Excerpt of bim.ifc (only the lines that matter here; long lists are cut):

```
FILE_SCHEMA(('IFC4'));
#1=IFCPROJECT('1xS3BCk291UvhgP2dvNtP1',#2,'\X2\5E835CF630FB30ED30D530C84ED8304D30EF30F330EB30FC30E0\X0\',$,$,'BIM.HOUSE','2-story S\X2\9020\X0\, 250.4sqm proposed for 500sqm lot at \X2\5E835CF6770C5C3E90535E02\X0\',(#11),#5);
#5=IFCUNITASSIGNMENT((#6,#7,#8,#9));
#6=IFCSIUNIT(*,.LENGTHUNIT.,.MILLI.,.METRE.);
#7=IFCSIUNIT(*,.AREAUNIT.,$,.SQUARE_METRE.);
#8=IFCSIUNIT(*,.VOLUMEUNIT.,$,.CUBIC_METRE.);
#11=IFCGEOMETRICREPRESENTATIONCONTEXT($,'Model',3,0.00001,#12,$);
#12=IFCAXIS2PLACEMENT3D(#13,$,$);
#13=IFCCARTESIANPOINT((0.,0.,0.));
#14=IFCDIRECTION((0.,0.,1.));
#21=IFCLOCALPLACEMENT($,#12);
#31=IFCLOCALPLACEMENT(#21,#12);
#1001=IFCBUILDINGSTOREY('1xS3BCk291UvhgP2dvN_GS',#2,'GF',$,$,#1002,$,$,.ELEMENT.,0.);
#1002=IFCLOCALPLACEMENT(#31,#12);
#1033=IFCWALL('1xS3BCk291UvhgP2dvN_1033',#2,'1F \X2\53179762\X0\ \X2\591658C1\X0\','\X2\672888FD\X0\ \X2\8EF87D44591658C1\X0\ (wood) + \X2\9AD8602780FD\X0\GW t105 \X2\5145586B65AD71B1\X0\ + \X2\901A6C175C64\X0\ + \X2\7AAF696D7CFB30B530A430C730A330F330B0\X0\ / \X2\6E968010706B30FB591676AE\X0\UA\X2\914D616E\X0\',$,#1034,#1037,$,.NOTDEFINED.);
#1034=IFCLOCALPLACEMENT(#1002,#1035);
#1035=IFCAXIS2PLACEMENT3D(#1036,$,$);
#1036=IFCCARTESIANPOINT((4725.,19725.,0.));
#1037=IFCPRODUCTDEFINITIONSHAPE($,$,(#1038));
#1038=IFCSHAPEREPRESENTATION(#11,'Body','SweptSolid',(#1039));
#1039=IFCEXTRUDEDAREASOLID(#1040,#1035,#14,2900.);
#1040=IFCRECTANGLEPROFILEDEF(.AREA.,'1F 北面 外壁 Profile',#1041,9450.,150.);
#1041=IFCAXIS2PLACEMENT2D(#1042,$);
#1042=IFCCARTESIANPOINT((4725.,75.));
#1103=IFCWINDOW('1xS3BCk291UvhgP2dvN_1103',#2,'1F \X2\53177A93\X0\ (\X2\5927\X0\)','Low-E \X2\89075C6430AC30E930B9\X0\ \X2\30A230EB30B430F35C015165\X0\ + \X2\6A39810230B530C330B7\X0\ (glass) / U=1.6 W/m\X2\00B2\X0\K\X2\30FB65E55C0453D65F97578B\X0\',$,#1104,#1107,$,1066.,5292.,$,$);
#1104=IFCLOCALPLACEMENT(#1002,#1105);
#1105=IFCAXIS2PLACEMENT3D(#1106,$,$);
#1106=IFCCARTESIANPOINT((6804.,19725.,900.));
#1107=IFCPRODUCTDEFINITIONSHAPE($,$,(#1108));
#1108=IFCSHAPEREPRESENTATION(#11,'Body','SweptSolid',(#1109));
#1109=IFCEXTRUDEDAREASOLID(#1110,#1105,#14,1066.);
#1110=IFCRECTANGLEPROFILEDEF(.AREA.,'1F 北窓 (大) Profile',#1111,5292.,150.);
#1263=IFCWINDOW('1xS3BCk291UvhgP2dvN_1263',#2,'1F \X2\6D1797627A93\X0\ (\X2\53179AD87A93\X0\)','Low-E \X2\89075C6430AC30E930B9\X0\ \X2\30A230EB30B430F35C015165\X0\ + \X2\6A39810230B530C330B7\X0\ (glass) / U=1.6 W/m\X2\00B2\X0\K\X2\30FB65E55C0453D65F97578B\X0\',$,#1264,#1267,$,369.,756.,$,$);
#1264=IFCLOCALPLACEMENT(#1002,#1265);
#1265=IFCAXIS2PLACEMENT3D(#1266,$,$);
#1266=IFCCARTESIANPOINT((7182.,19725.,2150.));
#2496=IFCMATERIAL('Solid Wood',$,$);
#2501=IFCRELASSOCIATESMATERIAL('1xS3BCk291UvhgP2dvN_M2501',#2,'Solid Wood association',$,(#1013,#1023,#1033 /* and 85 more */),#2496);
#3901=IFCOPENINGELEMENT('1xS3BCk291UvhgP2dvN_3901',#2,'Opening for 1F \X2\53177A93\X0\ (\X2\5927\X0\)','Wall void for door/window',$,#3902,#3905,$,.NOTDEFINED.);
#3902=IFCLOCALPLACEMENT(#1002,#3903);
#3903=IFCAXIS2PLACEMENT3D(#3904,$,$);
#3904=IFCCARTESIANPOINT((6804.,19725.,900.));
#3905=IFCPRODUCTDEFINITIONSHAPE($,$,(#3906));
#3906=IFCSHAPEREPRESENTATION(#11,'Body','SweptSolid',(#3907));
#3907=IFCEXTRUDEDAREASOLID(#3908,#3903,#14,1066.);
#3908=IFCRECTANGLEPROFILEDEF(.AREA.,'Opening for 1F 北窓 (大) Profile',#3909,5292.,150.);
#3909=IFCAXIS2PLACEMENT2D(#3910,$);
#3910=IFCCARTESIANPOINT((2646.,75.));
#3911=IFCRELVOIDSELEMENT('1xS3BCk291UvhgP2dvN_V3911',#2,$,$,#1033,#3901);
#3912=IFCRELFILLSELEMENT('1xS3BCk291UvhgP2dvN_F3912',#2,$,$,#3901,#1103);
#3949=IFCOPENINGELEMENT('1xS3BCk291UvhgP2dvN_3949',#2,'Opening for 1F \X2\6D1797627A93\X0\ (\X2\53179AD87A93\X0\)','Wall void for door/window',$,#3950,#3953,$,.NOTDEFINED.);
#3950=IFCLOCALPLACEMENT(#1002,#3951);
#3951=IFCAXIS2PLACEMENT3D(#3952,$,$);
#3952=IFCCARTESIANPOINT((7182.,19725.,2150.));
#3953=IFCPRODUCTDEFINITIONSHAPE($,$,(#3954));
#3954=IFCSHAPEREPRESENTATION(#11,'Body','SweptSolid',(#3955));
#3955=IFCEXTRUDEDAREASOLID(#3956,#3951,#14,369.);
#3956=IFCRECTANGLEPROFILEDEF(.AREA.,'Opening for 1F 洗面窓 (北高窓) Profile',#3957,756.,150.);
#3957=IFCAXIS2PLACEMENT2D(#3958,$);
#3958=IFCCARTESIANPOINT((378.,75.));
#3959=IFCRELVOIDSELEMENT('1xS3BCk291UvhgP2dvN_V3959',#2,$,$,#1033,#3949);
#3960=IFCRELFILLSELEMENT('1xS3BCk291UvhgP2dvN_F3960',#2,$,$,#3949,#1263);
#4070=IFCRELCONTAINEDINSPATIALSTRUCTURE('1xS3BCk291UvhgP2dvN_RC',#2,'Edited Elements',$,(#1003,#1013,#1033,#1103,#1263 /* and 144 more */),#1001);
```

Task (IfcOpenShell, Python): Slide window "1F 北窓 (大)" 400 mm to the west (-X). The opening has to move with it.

```python
import ifcopenshell
import ifcopenshell.api.geometry
import ifcopenshell.util.placement

model = ifcopenshell.open("bim.ifc")

window = model.by_guid("1xS3BCk291UvhgP2dvN_1103")
opening = window.FillsVoids[0].RelatingOpeningElement
wall = opening.VoidsElements[0].RelatingBuildingElement

wall_matrix = ifcopenshell.util.placement.get_local_placement(wall.ObjectPlacement)
shift = wall_matrix[:3, 0] * -400.0
before = ifcopenshell.util.placement.get_local_placement(window.ObjectPlacement)[:3, 3].copy()

# The window is not placed relative to its opening, so move both.
for product in (opening, window):
    matrix = ifcopenshell.util.placement.get_local_placement(product.ObjectPlacement)
    matrix[:3, 3] += shift
    ifcopenshell.api.geometry.edit_object_placement(model, product=product, matrix=matrix, is_si=False)

after = ifcopenshell.util.placement.get_local_placement(window.ObjectPlacement)[:3, 3]
print("window moved by", (after - before).round(3) + 0.0)

model.write("bim-out.ifc")
```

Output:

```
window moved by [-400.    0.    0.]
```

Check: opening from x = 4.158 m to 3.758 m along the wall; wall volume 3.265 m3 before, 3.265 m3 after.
